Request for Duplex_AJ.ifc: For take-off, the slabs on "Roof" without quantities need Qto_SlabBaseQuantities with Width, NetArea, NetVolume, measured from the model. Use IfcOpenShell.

First a look at what the model holds.

```python
import ifcopenshell
import ifcopenshell.util.element
import ifcopenshell.util.unit

model = ifcopenshell.open("Duplex_AJ.ifc")
print(model.schema)
for unit_type in ("LENGTHUNIT", "AREAUNIT", "VOLUMEUNIT"):
    print(unit_type, ifcopenshell.util.unit.calculate_unit_scale(model, unit_type))
storey = next(s for s in model.by_type("IfcBuildingStorey") if s.Name == "Roof")
slabs = [e for e in ifcopenshell.util.element.get_decomposition(storey) if e.is_a("IfcSlab")]
for e in sorted(slabs, key=lambda e: e.id()):
    print(e.id(), e.is_a(), e.Name, list(ifcopenshell.util.element.get_psets(e, qtos_only=True)), sep=" | ")
```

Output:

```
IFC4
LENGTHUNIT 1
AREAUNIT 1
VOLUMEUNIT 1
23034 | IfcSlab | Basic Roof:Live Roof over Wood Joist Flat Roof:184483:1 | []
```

```python
import ifcopenshell
import ifcopenshell.api.pset
import ifcopenshell.geom
import ifcopenshell.util.element
import ifcopenshell.util.shape
import ifcopenshell.util.unit

model = ifcopenshell.open("Duplex_AJ.ifc")
unit_scale = ifcopenshell.util.unit.calculate_unit_scale(model)
area_scale = ifcopenshell.util.unit.calculate_unit_scale(model, "AREAUNIT")
volume_scale = ifcopenshell.util.unit.calculate_unit_scale(model, "VOLUMEUNIT")
settings = ifcopenshell.geom.settings()

storey = next(s for s in model.by_type("IfcBuildingStorey") if s.Name == "Roof")
slabs = [e for e in ifcopenshell.util.element.get_decomposition(storey) if e.is_a("IfcSlab")]

for e in sorted(slabs, key=lambda e: e.id()):
    if ifcopenshell.util.element.get_psets(e, qtos_only=True, should_inherit=False):
        continue
    # Geometry comes back in metres, in the element's own axes.
    shape = ifcopenshell.geom.create_shape(settings, e)
    values = {
        "Width": ifcopenshell.util.shape.get_z(shape.geometry) / unit_scale,
        "NetArea": ifcopenshell.util.shape.get_footprint_area(shape.geometry) / area_scale,
        "NetVolume": ifcopenshell.util.shape.get_volume(shape.geometry) / volume_scale,
    }
    qto = ifcopenshell.api.pset.add_qto(model, product=e, name="Qto_SlabBaseQuantities")
    ifcopenshell.api.pset.edit_qto(model, qto=qto, properties=values)
    print(e.id(), {k: round(v, 3) for k, v in values.items()})

model.write("Duplex_AJ_edited.ifc")
```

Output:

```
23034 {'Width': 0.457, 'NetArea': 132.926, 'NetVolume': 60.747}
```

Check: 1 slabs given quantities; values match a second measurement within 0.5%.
